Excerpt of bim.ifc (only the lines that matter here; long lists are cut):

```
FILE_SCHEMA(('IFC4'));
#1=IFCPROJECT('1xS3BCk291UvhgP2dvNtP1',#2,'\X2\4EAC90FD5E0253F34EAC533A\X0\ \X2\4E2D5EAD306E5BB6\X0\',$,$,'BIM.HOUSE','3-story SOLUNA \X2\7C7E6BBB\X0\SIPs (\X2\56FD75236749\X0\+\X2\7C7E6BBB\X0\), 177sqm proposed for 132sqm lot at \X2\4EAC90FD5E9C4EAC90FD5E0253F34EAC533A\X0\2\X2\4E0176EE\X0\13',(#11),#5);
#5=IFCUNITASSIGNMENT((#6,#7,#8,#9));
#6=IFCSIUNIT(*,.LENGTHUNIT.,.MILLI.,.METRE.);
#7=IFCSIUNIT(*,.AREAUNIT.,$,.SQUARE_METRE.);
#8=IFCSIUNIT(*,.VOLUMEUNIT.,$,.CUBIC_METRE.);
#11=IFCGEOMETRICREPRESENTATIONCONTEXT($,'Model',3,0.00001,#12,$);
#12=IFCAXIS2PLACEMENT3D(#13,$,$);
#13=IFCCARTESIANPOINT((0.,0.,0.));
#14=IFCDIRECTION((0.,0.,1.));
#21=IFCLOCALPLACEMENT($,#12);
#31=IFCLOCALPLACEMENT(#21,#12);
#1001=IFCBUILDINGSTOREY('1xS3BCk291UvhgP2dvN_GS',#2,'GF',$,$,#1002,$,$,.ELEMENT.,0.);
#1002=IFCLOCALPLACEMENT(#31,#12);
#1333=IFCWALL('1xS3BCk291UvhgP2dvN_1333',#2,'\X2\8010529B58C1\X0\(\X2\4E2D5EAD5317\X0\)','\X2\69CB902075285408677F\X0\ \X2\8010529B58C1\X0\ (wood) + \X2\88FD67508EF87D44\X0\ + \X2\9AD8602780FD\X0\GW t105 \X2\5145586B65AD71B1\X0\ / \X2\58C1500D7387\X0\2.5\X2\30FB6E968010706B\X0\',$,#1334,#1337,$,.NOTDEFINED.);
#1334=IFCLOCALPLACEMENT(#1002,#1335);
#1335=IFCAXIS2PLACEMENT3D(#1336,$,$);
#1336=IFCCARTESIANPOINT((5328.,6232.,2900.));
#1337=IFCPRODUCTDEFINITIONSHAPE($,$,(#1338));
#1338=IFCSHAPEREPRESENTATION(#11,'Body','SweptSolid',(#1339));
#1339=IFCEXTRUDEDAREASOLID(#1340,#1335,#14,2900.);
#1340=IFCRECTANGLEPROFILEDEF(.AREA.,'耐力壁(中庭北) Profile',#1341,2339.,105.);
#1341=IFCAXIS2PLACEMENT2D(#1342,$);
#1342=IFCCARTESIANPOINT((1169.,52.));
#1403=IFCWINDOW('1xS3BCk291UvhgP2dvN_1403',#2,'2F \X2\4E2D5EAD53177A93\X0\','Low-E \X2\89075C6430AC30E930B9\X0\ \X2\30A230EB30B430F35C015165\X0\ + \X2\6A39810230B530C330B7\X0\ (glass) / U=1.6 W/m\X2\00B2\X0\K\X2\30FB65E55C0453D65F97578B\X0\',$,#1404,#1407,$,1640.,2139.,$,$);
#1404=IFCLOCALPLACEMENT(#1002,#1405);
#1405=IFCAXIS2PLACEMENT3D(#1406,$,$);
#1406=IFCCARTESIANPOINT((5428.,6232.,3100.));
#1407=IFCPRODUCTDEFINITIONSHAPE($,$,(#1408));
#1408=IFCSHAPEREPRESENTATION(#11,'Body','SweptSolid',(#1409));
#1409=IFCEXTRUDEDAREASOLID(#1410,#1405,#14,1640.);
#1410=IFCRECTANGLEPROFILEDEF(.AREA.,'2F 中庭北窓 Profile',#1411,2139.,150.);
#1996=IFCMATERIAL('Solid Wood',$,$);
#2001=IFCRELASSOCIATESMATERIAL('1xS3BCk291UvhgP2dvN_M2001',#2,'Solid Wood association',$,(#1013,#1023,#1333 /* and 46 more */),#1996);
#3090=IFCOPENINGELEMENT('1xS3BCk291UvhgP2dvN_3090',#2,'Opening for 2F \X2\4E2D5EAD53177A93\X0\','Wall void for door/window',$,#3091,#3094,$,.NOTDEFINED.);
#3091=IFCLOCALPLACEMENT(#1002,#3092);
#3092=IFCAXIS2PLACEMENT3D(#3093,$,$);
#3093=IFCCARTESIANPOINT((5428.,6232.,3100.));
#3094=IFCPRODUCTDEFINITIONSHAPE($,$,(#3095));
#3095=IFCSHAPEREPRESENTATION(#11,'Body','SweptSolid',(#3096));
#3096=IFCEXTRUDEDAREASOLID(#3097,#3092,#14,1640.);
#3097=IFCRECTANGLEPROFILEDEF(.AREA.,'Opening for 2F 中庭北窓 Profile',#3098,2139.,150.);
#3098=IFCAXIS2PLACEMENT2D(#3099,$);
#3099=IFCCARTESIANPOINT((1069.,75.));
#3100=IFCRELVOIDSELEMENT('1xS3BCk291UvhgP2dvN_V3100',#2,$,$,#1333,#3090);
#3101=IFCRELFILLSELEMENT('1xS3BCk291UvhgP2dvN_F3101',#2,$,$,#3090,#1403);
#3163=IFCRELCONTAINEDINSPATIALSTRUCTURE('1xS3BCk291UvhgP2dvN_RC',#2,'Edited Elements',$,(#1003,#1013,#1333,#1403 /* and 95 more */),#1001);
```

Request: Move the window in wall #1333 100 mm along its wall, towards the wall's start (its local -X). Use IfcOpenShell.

```python
import ifcopenshell
import ifcopenshell.api.geometry
import ifcopenshell.util.placement

model = ifcopenshell.open("bim.ifc")

window = model.by_id(1403)
opening = window.FillsVoids[0].RelatingOpeningElement
wall = opening.VoidsElements[0].RelatingBuildingElement

wall_matrix = ifcopenshell.util.placement.get_local_placement(wall.ObjectPlacement)
shift = wall_matrix[:3, 0] * -100.0
before = ifcopenshell.util.placement.get_local_placement(window.ObjectPlacement)[:3, 3].copy()

# The window is not placed relative to its opening, so move both.
for product in (opening, window):
    matrix = ifcopenshell.util.placement.get_local_placement(product.ObjectPlacement)
    matrix[:3, 3] += shift
    ifcopenshell.api.geometry.edit_object_placement(model, product=product, matrix=matrix, is_si=False)

after = ifcopenshell.util.placement.get_local_placement(window.ObjectPlacement)[:3, 3]
print("window moved by", (after - before).round(3) + 0.0)

model.write("bim_v2.ifc")
```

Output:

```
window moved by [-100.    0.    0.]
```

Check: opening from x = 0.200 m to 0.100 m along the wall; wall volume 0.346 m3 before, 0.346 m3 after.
